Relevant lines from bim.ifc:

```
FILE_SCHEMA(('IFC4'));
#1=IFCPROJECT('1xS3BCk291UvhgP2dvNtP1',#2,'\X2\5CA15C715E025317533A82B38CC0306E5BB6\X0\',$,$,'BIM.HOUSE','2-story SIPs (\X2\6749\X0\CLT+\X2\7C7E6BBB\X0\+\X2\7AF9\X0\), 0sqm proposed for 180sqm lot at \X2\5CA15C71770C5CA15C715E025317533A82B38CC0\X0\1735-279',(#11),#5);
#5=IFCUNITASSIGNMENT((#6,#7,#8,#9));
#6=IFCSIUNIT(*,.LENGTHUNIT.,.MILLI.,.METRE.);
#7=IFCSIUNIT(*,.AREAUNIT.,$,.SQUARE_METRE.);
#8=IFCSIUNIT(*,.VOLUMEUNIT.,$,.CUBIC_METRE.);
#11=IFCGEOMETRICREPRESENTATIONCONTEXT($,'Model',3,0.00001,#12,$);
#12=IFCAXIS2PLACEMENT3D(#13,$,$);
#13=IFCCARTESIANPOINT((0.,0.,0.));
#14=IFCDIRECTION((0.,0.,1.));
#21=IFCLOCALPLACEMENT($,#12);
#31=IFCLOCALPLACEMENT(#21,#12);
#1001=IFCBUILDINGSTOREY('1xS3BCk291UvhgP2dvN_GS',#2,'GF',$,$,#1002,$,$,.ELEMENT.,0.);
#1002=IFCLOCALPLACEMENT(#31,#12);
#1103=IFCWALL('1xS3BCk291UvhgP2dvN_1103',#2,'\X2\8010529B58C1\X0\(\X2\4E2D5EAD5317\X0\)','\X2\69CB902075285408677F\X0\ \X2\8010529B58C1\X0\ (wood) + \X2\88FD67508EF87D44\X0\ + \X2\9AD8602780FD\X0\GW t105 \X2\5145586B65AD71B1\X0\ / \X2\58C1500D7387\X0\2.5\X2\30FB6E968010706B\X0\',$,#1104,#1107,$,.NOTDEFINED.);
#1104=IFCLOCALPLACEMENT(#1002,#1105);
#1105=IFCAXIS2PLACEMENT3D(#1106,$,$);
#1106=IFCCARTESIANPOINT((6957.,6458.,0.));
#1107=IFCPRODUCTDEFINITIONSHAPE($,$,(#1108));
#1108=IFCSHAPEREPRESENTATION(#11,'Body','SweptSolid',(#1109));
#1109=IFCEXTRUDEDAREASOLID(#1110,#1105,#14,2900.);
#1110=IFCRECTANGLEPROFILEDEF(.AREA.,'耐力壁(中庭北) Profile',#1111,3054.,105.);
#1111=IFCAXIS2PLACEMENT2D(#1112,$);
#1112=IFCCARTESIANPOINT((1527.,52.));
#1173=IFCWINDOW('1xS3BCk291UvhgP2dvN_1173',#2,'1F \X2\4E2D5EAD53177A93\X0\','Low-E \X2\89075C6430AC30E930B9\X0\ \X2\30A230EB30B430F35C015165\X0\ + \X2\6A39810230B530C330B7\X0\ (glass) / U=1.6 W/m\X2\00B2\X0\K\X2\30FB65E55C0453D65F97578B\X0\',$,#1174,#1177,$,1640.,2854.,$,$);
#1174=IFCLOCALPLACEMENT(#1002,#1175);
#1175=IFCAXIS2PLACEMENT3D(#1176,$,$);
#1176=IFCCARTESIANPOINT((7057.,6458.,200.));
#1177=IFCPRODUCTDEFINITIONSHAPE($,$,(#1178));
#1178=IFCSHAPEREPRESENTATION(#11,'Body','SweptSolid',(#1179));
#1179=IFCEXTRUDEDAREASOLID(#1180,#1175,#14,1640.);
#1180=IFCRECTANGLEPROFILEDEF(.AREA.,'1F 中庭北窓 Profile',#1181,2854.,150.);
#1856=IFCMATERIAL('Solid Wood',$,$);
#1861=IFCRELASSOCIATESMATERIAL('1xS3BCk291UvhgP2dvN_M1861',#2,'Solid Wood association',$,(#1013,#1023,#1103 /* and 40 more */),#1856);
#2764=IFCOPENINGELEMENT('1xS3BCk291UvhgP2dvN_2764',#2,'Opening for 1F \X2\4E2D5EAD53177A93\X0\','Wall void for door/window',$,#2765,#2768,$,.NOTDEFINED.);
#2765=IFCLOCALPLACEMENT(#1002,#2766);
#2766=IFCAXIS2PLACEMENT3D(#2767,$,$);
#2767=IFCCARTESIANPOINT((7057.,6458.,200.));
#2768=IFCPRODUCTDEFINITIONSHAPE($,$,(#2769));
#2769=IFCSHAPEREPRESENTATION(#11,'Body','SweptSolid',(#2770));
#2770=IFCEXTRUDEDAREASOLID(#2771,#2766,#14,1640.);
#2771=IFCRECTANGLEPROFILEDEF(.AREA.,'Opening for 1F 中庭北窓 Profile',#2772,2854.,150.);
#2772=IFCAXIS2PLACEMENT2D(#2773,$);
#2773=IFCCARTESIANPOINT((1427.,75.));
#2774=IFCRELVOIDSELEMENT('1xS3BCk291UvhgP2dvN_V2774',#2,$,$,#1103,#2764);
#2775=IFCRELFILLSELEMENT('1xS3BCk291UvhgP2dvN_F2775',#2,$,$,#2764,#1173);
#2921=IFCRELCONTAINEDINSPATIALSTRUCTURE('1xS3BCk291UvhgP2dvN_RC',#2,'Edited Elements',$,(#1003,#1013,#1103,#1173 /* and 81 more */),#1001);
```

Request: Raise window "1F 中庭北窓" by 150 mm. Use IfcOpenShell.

```python
import numpy as np
import ifcopenshell
import ifcopenshell.api.geometry
import ifcopenshell.util.placement
import ifcopenshell.util.unit

model = ifcopenshell.open("bim.ifc")
unit_scale = ifcopenshell.util.unit.calculate_unit_scale(model)

window = model.by_id(1173)
opening = window.FillsVoids[0].RelatingOpeningElement
dz = 0.15 / unit_scale

shift = np.array([0.0, 0.0, dz])
# The window is not placed relative to its opening, so move both.
for product in (opening, window):
    matrix = ifcopenshell.util.placement.get_local_placement(product.ObjectPlacement)
    matrix[:3, 3] += shift
    ifcopenshell.api.geometry.edit_object_placement(model, product=product, matrix=matrix, is_si=False)

print(f"moved by {dz * unit_scale:+.3f} m")

model.write("bim-out.ifc")
```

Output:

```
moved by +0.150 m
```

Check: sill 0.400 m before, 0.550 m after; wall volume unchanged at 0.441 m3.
